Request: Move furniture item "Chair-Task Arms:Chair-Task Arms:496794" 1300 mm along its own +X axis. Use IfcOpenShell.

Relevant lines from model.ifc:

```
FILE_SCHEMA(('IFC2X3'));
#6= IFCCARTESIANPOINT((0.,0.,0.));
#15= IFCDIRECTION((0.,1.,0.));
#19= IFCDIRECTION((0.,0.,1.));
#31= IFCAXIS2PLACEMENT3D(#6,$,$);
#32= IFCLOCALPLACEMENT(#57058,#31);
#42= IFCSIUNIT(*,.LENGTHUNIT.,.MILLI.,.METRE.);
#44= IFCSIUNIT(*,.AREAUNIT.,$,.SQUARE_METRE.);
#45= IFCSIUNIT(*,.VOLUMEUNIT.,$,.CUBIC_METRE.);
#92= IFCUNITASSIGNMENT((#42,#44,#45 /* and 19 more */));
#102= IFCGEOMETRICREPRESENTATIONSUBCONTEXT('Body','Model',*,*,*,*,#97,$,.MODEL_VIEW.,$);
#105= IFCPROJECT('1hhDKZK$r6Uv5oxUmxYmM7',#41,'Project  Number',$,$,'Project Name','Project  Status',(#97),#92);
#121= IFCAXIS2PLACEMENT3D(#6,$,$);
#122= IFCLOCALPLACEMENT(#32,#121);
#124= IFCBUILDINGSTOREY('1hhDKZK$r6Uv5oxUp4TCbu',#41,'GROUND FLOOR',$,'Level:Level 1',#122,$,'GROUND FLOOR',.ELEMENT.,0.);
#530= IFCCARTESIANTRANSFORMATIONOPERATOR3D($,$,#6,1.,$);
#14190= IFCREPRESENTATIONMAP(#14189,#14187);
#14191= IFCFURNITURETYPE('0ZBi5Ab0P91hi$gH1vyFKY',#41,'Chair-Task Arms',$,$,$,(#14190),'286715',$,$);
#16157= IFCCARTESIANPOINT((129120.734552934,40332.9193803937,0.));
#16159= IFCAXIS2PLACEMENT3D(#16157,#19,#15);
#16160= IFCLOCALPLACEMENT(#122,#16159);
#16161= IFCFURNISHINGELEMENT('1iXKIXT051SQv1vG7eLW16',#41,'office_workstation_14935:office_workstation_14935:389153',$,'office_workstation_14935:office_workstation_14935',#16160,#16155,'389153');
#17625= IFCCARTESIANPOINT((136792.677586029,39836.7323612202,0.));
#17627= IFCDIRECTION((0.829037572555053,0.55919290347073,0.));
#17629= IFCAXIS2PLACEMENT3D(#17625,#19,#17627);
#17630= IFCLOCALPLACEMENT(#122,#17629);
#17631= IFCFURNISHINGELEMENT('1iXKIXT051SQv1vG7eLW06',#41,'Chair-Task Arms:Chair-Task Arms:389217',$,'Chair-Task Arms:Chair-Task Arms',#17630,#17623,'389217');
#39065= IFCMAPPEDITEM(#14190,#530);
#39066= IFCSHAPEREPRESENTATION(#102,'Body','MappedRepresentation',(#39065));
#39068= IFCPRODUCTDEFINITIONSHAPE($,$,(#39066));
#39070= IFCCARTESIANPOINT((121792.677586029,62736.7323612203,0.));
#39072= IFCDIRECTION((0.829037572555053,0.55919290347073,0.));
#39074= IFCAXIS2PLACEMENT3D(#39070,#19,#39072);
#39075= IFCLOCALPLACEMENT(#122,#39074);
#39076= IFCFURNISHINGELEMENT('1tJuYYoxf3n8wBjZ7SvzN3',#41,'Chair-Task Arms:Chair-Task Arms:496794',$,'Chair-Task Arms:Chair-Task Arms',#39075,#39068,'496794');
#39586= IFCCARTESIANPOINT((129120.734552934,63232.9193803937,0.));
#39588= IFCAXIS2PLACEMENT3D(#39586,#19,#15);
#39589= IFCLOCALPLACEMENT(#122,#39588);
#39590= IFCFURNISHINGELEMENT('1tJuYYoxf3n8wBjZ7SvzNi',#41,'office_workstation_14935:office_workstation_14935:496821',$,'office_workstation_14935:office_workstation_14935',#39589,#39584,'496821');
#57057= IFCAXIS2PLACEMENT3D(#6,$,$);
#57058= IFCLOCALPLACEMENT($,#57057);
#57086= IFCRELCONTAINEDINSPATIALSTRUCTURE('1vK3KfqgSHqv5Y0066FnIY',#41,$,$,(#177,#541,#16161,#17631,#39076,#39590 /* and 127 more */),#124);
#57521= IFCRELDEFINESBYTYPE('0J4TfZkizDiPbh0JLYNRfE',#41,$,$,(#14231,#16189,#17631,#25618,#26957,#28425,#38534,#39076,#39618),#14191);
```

```python
import ifcopenshell
import ifcopenshell.api.geometry
import ifcopenshell.util.placement
import ifcopenshell.util.unit

model = ifcopenshell.open("model.ifc")
unit_scale = ifcopenshell.util.unit.calculate_unit_scale(model)

item = model.by_guid("1tJuYYoxf3n8wBjZ7SvzN3")
matrix = ifcopenshell.util.placement.get_local_placement(item.ObjectPlacement)
matrix[:3, 3] += matrix[:3, 0] * 1.3 / unit_scale
ifcopenshell.api.geometry.edit_object_placement(model, product=item, matrix=matrix, is_si=False)

print(ifcopenshell.util.placement.get_local_placement(item.ObjectPlacement).round(3) + 0.0)

model.write("model_rev.ifc")
```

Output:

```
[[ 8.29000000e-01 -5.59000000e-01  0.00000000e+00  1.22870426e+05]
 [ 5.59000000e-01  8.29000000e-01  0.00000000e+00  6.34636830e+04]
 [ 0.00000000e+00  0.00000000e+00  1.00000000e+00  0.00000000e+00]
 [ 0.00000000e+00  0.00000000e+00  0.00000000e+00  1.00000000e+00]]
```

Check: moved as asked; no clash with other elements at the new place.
